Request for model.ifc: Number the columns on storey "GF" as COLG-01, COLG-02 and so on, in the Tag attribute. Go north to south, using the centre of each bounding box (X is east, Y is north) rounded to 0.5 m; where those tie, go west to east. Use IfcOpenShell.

First a look at what the model holds.

```python
import ifcopenshell
import ifcopenshell.util.element
import ifcopenshell.util.placement

model = ifcopenshell.open("model.ifc")
print(model.schema)
storey = next(s for s in model.by_type("IfcBuildingStorey") if s.Name == "GF")
columns = [e for e in ifcopenshell.util.element.get_decomposition(storey) if e.is_a("IfcColumn")]
for e in sorted(columns, key=lambda e: e.id()):
    origin = ifcopenshell.util.placement.get_local_placement(e.ObjectPlacement)[:3, 3]
    print(e.id(), e.Tag, e.Name, origin.round(2) + 0.0, sep=" | ")
```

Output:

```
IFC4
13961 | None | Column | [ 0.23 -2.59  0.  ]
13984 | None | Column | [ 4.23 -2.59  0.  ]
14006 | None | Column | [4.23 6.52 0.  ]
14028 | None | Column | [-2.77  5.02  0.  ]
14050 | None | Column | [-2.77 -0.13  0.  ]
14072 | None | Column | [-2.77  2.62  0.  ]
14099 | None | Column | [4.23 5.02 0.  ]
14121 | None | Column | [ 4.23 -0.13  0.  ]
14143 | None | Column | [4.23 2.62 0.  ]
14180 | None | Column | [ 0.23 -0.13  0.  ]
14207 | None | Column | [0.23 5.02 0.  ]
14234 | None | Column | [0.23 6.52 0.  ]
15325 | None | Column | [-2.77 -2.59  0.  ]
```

```python
import ifcopenshell
import ifcopenshell.geom
import ifcopenshell.util.element
import ifcopenshell.util.shape

model = ifcopenshell.open("model.ifc")
settings = ifcopenshell.geom.settings()
settings.set("use-world-coords", True)


def centre(element):
    shape = ifcopenshell.geom.create_shape(settings, element)
    return ifcopenshell.util.shape.get_bbox_centroid(shape.geometry)


storey = next(s for s in model.by_type("IfcBuildingStorey") if s.Name == "GF")
columns = [e for e in ifcopenshell.util.element.get_decomposition(storey) if e.is_a("IfcColumn")]

# Insertion points can sit at a corner or the storey origin, so sort by the geometry (in metres).
centres = {e: centre(e) for e in columns}
columns.sort(key=lambda e: (-round(centres[e][1] / 0.5), centres[e][0]))

for i, e in enumerate(columns, start=1):
    number = f"COLG-{i:02d}"
    e.Tag = number
    print(e.id(), number)

model.write("model_edited.ifc")
```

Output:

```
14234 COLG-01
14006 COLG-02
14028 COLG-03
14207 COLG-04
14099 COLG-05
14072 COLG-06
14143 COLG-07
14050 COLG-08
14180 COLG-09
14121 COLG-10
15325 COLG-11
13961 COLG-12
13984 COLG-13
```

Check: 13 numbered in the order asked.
